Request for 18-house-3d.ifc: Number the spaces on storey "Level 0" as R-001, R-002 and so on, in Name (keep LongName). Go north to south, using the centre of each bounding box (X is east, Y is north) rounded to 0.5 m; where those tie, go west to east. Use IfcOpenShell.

First a look at what the model holds.

```python
import ifcopenshell
import ifcopenshell.util.element
import ifcopenshell.util.placement

model = ifcopenshell.open("18-house-3d.ifc")
print(model.schema)
storey = next(s for s in model.by_type("IfcBuildingStorey") if s.Name == "Level 0")
spaces = [e for e in ifcopenshell.util.element.get_decomposition(storey) if e.is_a("IfcSpace")]
for e in sorted(spaces, key=lambda e: e.id()):
    origin = ifcopenshell.util.placement.get_local_placement(e.ObjectPlacement)[:3, 3]
    print(e.id(), e.Name, e.LongName, origin.round(2) + 0.0, sep=" | ")
```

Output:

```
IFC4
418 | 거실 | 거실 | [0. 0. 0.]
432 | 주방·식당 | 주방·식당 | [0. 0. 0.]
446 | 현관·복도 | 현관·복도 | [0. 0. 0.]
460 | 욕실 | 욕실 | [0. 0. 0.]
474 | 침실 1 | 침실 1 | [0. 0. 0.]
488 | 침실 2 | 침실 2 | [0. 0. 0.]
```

```python
import ifcopenshell
import ifcopenshell.geom
import ifcopenshell.util.element
import ifcopenshell.util.shape

model = ifcopenshell.open("18-house-3d.ifc")
settings = ifcopenshell.geom.settings()
settings.set("use-world-coords", True)


def centre(element):
    shape = ifcopenshell.geom.create_shape(settings, element)
    return ifcopenshell.util.shape.get_bbox_centroid(shape.geometry)


storey = next(s for s in model.by_type("IfcBuildingStorey") if s.Name == "Level 0")
spaces = [e for e in ifcopenshell.util.element.get_decomposition(storey) if e.is_a("IfcSpace")]

# Insertion points can sit at a corner or the storey origin, so sort by the geometry (in metres).
centres = {e: centre(e) for e in spaces}
spaces.sort(key=lambda e: (-round(centres[e][1] / 0.5), centres[e][0]))

for i, e in enumerate(spaces, start=1):
    number = f"R-0{i:02d}"
    e.Name = number
    print(e.id(), number)

model.write("18-house-3d_edited.ifc")
```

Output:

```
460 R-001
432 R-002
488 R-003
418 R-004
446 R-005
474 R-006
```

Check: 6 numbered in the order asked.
